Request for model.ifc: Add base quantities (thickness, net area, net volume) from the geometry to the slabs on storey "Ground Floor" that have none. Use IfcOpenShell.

First a look at what the model holds.

```python
import ifcopenshell
import ifcopenshell.util.element
import ifcopenshell.util.unit

model = ifcopenshell.open("model.ifc")
print(model.schema)
for unit_type in ("LENGTHUNIT", "AREAUNIT", "VOLUMEUNIT"):
    print(unit_type, ifcopenshell.util.unit.calculate_unit_scale(model, unit_type))
storey = next(s for s in model.by_type("IfcBuildingStorey") if s.Name == "Ground Floor")
slabs = [e for e in ifcopenshell.util.element.get_decomposition(storey) if e.is_a("IfcSlab")]
for e in sorted(slabs, key=lambda e: e.id()):
    print(e.id(), e.is_a(), e.Name, list(ifcopenshell.util.element.get_psets(e, qtos_only=True)), sep=" | ")
```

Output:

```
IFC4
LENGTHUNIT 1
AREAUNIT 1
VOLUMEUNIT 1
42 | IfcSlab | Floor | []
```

```python
import ifcopenshell
import ifcopenshell.api.pset
import ifcopenshell.geom
import ifcopenshell.util.element
import ifcopenshell.util.shape
import ifcopenshell.util.unit

model = ifcopenshell.open("model.ifc")
unit_scale = ifcopenshell.util.unit.calculate_unit_scale(model)
area_scale = ifcopenshell.util.unit.calculate_unit_scale(model, "AREAUNIT")
volume_scale = ifcopenshell.util.unit.calculate_unit_scale(model, "VOLUMEUNIT")
settings = ifcopenshell.geom.settings()

storey = next(s for s in model.by_type("IfcBuildingStorey") if s.Name == "Ground Floor")
slabs = [e for e in ifcopenshell.util.element.get_decomposition(storey) if e.is_a("IfcSlab")]

for e in sorted(slabs, key=lambda e: e.id()):
    if ifcopenshell.util.element.get_psets(e, qtos_only=True, should_inherit=False):
        continue
    # Geometry comes back in metres, in the element's own axes.
    shape = ifcopenshell.geom.create_shape(settings, e)
    values = {
        "Width": ifcopenshell.util.shape.get_z(shape.geometry) / unit_scale,
        "NetArea": ifcopenshell.util.shape.get_footprint_area(shape.geometry) / area_scale,
        "NetVolume": ifcopenshell.util.shape.get_volume(shape.geometry) / volume_scale,
    }
    qto = ifcopenshell.api.pset.add_qto(model, product=e, name="Qto_SlabBaseQuantities")
    ifcopenshell.api.pset.edit_qto(model, qto=qto, properties=values)
    print(e.id(), {k: round(v, 3) for k, v in values.items()})

model.write("model_rev.ifc")
```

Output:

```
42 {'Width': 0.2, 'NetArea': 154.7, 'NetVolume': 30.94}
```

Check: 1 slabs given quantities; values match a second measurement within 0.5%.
